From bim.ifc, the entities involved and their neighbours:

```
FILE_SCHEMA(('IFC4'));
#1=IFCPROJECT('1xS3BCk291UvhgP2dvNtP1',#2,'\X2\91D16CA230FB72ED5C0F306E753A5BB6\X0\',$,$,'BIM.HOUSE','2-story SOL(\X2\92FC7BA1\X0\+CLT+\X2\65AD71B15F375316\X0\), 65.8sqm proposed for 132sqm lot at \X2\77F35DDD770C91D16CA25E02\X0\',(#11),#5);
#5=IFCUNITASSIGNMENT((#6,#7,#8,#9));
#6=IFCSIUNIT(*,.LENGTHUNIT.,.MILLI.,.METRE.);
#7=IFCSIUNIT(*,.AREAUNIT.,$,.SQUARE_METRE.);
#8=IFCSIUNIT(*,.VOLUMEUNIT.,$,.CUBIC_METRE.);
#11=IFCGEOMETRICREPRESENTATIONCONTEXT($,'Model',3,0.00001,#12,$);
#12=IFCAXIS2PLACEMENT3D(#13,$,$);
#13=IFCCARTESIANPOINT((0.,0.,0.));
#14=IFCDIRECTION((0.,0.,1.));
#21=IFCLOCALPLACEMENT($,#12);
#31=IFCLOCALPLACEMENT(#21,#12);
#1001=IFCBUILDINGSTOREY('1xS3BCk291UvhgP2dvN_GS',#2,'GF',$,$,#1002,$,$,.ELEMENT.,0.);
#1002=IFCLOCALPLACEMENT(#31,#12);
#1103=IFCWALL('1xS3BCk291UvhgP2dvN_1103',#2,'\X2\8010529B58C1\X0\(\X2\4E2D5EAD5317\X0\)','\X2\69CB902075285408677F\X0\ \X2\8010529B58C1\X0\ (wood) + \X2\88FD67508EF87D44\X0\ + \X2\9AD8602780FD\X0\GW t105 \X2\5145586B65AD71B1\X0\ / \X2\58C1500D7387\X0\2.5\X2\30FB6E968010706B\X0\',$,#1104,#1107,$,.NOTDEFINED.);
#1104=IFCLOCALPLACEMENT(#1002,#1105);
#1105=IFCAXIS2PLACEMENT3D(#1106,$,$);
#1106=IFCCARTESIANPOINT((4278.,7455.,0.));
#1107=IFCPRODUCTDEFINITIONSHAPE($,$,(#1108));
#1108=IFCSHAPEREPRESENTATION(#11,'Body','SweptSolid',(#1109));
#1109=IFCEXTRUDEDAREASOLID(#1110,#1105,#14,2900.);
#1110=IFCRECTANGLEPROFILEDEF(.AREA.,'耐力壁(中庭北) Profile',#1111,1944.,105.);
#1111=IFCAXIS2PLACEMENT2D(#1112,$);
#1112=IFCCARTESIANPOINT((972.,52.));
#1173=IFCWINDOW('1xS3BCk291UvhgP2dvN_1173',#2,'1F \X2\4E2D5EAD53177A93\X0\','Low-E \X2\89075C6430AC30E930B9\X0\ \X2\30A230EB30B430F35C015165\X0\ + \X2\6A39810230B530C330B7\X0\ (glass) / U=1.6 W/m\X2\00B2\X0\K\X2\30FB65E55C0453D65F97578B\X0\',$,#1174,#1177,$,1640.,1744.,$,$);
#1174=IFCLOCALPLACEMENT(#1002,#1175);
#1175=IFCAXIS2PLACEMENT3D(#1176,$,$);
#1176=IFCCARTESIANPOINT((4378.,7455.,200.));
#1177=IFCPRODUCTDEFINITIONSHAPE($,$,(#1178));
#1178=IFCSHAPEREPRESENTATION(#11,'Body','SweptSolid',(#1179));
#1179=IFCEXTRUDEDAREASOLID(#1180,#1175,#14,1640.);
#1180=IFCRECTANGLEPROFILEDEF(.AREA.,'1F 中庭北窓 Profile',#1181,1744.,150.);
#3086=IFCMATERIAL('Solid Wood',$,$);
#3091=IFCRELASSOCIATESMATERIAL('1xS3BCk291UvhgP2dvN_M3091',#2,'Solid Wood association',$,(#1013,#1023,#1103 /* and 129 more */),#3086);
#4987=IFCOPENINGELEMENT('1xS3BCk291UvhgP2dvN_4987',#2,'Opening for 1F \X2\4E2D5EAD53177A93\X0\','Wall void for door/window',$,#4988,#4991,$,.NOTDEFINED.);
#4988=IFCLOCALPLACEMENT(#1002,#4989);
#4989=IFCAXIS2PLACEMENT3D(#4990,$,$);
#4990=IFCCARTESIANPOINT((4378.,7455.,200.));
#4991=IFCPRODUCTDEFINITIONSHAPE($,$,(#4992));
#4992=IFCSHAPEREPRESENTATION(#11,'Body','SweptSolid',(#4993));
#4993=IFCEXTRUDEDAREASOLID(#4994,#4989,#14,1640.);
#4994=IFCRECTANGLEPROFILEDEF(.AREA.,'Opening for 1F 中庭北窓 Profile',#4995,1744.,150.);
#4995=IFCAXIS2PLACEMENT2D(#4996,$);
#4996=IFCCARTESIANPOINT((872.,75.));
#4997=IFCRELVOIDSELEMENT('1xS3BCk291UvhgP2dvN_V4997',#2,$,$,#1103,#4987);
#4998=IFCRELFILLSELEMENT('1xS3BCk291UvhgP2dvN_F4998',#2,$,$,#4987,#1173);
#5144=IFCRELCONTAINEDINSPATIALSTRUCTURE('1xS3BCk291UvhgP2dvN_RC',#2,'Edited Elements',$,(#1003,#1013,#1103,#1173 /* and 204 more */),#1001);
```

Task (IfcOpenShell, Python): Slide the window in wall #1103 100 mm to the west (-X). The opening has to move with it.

```python
import ifcopenshell
import ifcopenshell.api.geometry
import ifcopenshell.util.placement
import ifcopenshell.util.unit

model = ifcopenshell.open("bim.ifc")
unit_scale = ifcopenshell.util.unit.calculate_unit_scale(model)

window = model.by_guid("1xS3BCk291UvhgP2dvN_1173")
opening = window.FillsVoids[0].RelatingOpeningElement
wall = opening.VoidsElements[0].RelatingBuildingElement

wall_matrix = ifcopenshell.util.placement.get_local_placement(wall.ObjectPlacement)
shift = wall_matrix[:3, 0] * -0.1 / unit_scale
before = ifcopenshell.util.placement.get_local_placement(window.ObjectPlacement)[:3, 3].copy()

# The window is not placed relative to its opening, so move both.
for product in (opening, window):
    matrix = ifcopenshell.util.placement.get_local_placement(product.ObjectPlacement)
    matrix[:3, 3] += shift
    ifcopenshell.api.geometry.edit_object_placement(model, product=product, matrix=matrix, is_si=False)

after = ifcopenshell.util.placement.get_local_placement(window.ObjectPlacement)[:3, 3]
print("window moved by", (after - before).round(3) + 0.0)

model.write("bim-out.ifc")
```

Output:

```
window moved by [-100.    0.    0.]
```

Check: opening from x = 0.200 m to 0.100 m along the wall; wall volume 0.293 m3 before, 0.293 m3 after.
